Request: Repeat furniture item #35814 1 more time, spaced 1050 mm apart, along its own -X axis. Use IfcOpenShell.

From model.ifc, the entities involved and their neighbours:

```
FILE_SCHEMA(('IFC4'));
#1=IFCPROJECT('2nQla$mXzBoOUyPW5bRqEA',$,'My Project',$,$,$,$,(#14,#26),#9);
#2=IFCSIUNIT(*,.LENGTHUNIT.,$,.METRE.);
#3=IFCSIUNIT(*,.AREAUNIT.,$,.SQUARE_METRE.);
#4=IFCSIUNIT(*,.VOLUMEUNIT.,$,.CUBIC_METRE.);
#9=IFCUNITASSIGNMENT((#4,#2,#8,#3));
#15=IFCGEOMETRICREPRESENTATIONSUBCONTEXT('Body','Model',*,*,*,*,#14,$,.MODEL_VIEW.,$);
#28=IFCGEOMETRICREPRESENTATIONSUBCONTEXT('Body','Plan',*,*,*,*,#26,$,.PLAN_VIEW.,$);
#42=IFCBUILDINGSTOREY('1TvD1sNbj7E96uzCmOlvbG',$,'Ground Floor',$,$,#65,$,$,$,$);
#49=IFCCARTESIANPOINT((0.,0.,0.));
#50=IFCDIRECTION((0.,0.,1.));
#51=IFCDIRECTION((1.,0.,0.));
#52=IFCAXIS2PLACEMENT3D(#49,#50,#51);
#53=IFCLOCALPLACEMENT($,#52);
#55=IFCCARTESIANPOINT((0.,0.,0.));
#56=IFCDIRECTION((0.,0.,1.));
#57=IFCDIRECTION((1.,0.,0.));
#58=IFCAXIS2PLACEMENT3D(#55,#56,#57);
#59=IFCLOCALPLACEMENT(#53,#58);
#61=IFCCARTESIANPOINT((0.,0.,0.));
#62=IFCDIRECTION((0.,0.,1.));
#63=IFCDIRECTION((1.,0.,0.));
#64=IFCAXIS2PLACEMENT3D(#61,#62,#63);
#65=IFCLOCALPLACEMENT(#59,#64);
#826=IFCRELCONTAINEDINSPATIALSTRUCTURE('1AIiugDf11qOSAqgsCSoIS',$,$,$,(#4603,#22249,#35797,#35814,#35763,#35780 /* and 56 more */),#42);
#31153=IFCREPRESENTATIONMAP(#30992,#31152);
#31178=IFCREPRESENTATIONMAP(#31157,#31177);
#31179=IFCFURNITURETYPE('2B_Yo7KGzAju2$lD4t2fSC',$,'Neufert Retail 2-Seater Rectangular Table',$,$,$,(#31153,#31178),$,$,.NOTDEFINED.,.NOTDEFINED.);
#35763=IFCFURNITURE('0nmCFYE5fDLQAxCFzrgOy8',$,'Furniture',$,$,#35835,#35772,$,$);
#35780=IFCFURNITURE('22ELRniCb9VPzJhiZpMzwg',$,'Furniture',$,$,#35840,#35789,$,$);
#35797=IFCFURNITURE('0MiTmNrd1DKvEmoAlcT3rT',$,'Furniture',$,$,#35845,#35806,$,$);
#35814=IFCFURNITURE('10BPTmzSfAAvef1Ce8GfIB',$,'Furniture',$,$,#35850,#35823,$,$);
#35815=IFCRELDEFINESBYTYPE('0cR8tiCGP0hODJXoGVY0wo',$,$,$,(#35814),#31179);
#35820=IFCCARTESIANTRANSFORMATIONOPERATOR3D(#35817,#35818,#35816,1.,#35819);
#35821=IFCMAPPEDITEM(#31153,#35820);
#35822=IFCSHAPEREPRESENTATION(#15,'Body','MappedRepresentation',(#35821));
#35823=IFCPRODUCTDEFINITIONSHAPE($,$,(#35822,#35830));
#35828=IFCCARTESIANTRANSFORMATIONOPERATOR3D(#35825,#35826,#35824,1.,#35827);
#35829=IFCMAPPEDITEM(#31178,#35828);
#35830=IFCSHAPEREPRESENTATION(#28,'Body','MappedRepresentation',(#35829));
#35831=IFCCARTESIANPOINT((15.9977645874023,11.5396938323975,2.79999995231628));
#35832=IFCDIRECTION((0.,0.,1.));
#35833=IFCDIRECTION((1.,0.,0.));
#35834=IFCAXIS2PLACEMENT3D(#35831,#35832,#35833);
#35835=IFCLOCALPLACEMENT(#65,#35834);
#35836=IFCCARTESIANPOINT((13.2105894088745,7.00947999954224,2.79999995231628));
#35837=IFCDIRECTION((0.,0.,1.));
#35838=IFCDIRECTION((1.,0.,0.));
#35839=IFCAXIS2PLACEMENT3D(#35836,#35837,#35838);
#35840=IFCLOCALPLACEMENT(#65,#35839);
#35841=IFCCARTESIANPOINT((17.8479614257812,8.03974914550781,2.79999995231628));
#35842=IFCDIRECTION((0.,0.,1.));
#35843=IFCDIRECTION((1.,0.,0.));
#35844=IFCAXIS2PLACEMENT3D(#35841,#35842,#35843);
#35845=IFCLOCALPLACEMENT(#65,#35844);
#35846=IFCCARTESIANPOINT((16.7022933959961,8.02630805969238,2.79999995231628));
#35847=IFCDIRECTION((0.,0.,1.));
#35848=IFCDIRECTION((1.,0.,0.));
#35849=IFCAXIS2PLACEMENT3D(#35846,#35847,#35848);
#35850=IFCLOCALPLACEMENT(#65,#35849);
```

```python
import ifcopenshell
import ifcopenshell.api.geometry
import ifcopenshell.api.root
import ifcopenshell.util.element
import ifcopenshell.util.placement
import ifcopenshell.util.unit

model = ifcopenshell.open("model.ifc")
unit_scale = ifcopenshell.util.unit.calculate_unit_scale(model)

source = model.by_guid("10BPTmzSfAAvef1Ce8GfIB")
base = ifcopenshell.util.placement.get_local_placement(source.ObjectPlacement)
step = -base[:3, 0] * 1.05 / unit_scale

for i in range(1, 2):
    copy = ifcopenshell.api.root.copy_class(model, product=source)
    copy.Representation = ifcopenshell.util.element.copy_deep(
        model, source.Representation, exclude=["IfcGeometricRepresentationContext", "IfcRepresentationMap"]
    )
    matrix = base.copy()
    matrix[:3, 3] += i * step
    print("added at", matrix[:3, 3].round(3) + 0.0)
    ifcopenshell.api.geometry.edit_object_placement(model, product=copy, matrix=matrix, is_si=False)

model.write("model_v2.ifc")
```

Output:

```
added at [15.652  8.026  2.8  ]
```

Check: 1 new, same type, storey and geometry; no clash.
